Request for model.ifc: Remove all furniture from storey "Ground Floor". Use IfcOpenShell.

First a look at what the model holds.

```python
import ifcopenshell
import ifcopenshell.util.element

model = ifcopenshell.open("model.ifc")
print(model.schema)
storey = next(s for s in model.by_type("IfcBuildingStorey") if s.Name == "Ground Floor")
furniture = [e for e in ifcopenshell.util.element.get_decomposition(storey) if e.is_a("IfcFurnishingElement")]
seen = {}
for e in furniture:
    element_type = ifcopenshell.util.element.get_type(e)
    name = element_type.Name if element_type not in (None, e) else None
    seen[name] = seen.get(name, 0) + 1
for name, count in sorted(seen.items(), key=str):
    print(count, "x", name)
```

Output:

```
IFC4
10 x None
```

```python
import ifcopenshell
import ifcopenshell.api.root
import ifcopenshell.util.element

model = ifcopenshell.open("model.ifc")

storey = next(s for s in model.by_type("IfcBuildingStorey") if s.Name == "Ground Floor")
furniture = [e for e in ifcopenshell.util.element.get_decomposition(storey) if e.is_a("IfcFurnishingElement")]

for e in furniture:
    ifcopenshell.api.root.remove_product(model, product=e)
print(len(furniture), "removed")

model.write("model_edited.ifc")
```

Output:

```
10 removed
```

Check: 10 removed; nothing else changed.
